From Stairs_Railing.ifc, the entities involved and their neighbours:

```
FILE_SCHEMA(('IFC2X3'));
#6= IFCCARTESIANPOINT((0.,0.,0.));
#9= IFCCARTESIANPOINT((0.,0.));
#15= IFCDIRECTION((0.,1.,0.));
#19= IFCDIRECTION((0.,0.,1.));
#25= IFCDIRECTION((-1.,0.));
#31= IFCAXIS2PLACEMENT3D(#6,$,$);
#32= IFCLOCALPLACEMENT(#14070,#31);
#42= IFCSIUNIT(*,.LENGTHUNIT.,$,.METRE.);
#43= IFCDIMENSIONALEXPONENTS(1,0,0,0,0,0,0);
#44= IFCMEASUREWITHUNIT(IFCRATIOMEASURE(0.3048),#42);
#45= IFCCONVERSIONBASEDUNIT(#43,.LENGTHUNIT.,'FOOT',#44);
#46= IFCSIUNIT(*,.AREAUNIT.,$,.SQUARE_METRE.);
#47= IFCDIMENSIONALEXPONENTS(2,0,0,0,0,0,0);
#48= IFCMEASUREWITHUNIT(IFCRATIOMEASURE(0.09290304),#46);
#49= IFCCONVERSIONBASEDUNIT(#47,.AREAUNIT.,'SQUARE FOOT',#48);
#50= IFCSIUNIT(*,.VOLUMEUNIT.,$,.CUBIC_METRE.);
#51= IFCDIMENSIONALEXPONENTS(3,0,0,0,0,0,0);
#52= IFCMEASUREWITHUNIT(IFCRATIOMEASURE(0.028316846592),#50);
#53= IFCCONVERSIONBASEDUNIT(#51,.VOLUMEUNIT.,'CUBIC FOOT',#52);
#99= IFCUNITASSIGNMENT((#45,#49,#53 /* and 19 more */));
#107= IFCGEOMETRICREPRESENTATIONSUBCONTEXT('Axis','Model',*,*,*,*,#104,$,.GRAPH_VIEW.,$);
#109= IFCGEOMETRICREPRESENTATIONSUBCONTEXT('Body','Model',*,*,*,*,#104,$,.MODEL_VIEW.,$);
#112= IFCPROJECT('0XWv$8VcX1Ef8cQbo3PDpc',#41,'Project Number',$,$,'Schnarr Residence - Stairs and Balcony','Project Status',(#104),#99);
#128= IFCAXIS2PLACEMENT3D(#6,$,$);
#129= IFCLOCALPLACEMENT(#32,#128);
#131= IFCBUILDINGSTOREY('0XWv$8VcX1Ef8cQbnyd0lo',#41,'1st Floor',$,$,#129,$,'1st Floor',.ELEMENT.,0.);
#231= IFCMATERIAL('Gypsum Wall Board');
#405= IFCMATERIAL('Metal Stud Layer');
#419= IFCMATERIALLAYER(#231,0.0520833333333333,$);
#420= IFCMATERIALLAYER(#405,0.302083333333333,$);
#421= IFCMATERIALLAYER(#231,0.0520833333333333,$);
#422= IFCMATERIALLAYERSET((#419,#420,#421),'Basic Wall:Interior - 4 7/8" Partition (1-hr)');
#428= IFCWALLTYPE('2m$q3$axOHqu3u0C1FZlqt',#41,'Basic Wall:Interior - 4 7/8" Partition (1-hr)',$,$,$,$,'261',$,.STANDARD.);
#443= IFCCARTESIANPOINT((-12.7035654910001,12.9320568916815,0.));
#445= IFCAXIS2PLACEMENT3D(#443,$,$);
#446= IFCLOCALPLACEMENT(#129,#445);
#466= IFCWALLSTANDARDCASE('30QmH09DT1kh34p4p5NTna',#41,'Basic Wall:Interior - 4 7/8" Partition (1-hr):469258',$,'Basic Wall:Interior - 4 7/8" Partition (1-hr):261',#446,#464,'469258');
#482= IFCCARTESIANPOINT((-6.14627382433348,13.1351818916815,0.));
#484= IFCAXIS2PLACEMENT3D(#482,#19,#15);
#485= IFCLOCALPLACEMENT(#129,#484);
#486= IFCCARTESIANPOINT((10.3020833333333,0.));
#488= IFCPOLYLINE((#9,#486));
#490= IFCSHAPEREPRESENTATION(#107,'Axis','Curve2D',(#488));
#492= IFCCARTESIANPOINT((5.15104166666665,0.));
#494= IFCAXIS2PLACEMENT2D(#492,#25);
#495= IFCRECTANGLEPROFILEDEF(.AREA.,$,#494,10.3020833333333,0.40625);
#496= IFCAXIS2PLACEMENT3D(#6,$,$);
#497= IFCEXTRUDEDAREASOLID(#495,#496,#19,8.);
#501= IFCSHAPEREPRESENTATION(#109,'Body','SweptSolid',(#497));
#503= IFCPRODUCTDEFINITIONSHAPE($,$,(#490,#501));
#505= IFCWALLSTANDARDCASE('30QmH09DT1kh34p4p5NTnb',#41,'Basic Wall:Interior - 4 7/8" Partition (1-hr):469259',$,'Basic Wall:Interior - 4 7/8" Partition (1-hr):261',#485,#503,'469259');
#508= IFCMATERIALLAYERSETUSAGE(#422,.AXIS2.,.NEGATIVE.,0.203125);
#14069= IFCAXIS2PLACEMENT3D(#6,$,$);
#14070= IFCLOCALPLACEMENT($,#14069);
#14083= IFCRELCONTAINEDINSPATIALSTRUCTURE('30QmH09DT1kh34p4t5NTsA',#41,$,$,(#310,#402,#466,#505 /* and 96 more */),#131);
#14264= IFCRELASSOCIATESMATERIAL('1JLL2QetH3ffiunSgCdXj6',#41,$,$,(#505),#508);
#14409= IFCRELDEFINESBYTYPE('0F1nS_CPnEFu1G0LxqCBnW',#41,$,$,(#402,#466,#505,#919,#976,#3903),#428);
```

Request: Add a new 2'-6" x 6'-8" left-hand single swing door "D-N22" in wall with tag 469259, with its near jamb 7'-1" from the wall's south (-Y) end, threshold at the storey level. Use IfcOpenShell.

```python
import numpy as np
import ifcopenshell
import ifcopenshell.api.feature
import ifcopenshell.api.geometry
import ifcopenshell.api.root
import ifcopenshell.api.spatial
import ifcopenshell.api.type
import ifcopenshell.geom
import ifcopenshell.util.element
import ifcopenshell.util.placement
import ifcopenshell.util.representation
import ifcopenshell.util.shape
import ifcopenshell.util.unit

model = ifcopenshell.open("Stairs_Railing.ifc")
unit_scale = ifcopenshell.util.unit.calculate_unit_scale(model)
settings = ifcopenshell.geom.settings()


def volume(element):
    """Net volume in cubic metres, openings subtracted."""
    shape = ifcopenshell.geom.create_shape(settings, element)
    return ifcopenshell.util.shape.get_volume(shape.geometry)


wall = model.by_guid("30QmH09DT1kh34p4p5NTnb")
storey = ifcopenshell.util.element.get_container(wall, ifc_class="IfcBuildingStorey")
context = ifcopenshell.util.representation.get_context(model, "Model", "Body", "MODEL_VIEW")
before = volume(wall)

width, height, from_end, sill = 0.762, 2.032, 2.159, 0.0  # metres

# The wall runs along its own X axis, and the end named is its -X end.
wall_shape = ifcopenshell.geom.create_shape(settings, wall)
x, y, z = ifcopenshell.util.shape.get_vertices(wall_shape.geometry).T
start = x.min() + from_end
face, thickness = float(y.min()), float(y.max() - y.min())
wall_matrix = ifcopenshell.util.placement.get_local_placement(wall.ObjectPlacement)
level = ifcopenshell.util.placement.get_local_placement(storey.ObjectPlacement)[2, 3]


def in_wall(x, y):
    """Placement at x, y metres in the wall's axes, at sill height."""
    matrix = wall_matrix.copy()
    matrix[:, 3] = wall_matrix @ np.array([x / unit_scale, y / unit_scale, 0.0, 1.0])
    matrix[2, 3] = level + sill / unit_scale
    return matrix


# Opening: a box that overshoots both wall faces by 50 mm.
opening = ifcopenshell.api.root.create_entity(model, ifc_class="IfcOpeningElement")
box = ifcopenshell.api.geometry.add_wall_representation(
    model, context=context, length=width, height=height, thickness=thickness + 0.1
)
ifcopenshell.api.geometry.assign_representation(model, product=opening, representation=box)
ifcopenshell.api.geometry.edit_object_placement(model, product=opening, matrix=in_wall(start, face - 0.05), is_si=False)
ifcopenshell.api.feature.add_feature(model, feature=opening, element=wall)

door = ifcopenshell.api.root.create_entity(model, ifc_class="IfcDoor", name="D-N22")
door.OverallWidth, door.OverallHeight = width / unit_scale, height / unit_scale
body = ifcopenshell.api.geometry.add_door_representation(
    model,
    context=context,
    overall_width=door.OverallWidth,
    overall_height=door.OverallHeight,
    operation_type="SINGLE_SWING_LEFT",
    lining_properties={"LiningDepth": thickness / unit_scale, "ThresholdDepth": thickness / unit_scale},
)
ifcopenshell.api.geometry.assign_representation(model, product=door, representation=body)
ifcopenshell.api.spatial.assign_container(model, products=[door], relating_structure=storey)
fills = ifcopenshell.api.feature.add_filling(model, opening=opening, element=door)
fills.OwnerHistory = door.OwnerHistory  # required in IFC2X3

# IFC2X3 keeps the operation on the door style.
style = ifcopenshell.api.root.create_entity(model, ifc_class="IfcDoorStyle", name="D-N22")
style.OperationType, style.ConstructionType = "SINGLE_SWING_LEFT", "NOTDEFINED"
style.ParameterTakesPrecedence = style.Sizeable = False
ifcopenshell.api.type.assign_type(model, related_objects=[door], relating_type=style)

# The lining spans the wall, so the door starts at the wall face.
ifcopenshell.api.geometry.edit_object_placement(model, product=door, matrix=in_wall(start, face), is_si=False)

after = volume(wall)

print(f"wall volume {before:.3f} -> {after:.3f} m3")

model.write("Stairs_Railing_v2.ifc")
```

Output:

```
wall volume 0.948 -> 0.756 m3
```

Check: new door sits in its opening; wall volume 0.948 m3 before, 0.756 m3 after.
